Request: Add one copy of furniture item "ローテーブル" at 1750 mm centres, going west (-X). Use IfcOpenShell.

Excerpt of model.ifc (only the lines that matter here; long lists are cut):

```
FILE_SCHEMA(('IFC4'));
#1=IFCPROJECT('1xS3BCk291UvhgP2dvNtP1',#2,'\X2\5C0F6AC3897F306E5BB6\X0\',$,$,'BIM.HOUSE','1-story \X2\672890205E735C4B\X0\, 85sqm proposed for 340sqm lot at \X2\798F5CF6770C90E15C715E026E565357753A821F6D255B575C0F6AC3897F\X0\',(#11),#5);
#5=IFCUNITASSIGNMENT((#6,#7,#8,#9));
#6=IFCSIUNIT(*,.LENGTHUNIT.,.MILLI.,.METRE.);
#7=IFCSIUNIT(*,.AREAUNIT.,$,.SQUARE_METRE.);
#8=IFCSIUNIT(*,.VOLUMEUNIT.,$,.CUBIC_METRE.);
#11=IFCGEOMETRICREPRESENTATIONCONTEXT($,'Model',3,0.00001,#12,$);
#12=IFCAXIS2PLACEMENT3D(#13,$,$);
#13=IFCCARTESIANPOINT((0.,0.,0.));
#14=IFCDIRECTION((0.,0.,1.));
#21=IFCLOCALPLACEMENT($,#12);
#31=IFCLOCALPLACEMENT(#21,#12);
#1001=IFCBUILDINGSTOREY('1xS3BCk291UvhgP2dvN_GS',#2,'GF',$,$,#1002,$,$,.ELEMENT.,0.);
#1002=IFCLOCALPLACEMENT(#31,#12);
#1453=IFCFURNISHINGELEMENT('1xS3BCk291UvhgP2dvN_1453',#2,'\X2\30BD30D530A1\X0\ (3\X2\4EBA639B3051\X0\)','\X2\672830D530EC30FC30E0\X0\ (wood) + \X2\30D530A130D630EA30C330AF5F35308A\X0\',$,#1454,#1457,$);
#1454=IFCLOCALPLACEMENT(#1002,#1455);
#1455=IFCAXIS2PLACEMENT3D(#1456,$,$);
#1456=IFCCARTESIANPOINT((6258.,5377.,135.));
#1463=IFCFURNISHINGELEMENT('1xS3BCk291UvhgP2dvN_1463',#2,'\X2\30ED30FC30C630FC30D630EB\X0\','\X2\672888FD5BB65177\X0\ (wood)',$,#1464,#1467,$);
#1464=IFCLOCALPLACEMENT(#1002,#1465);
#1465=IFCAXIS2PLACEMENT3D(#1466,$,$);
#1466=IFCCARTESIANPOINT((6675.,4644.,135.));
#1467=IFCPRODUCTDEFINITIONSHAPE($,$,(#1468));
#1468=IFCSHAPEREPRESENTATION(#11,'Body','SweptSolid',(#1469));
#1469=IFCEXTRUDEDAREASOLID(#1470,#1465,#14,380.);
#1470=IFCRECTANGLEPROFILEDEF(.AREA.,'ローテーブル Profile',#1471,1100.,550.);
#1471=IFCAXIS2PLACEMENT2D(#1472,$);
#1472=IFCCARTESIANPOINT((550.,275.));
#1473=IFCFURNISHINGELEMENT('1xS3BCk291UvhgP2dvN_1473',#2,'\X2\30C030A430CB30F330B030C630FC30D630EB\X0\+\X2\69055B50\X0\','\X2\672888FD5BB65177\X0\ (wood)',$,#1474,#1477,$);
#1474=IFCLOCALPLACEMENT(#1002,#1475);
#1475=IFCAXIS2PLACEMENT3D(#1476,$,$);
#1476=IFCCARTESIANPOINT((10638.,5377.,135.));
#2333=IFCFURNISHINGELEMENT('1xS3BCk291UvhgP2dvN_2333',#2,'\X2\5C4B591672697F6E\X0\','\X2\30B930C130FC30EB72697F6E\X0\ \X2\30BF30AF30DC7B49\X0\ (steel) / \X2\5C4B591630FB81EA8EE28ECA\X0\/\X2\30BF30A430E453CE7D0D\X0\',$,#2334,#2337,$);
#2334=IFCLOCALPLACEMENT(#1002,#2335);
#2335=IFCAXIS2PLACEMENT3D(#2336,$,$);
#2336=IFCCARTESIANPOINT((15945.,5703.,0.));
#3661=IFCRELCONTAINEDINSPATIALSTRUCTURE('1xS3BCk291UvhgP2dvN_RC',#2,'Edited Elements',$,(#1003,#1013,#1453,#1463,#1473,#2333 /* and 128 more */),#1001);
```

```python
import numpy as np
import ifcopenshell
import ifcopenshell.api.geometry
import ifcopenshell.api.root
import ifcopenshell.util.element
import ifcopenshell.util.placement
import ifcopenshell.util.unit

model = ifcopenshell.open("model.ifc")
unit_scale = ifcopenshell.util.unit.calculate_unit_scale(model)


def reuse_history(source, copy):
    """copy_class also copies each property set's owner history, people and application; keep the originals."""
    for rel in copy.IsDefinedBy:
        if rel.is_a("IfcRelDefinesByProperties") and (history := rel.RelatingPropertyDefinition.OwnerHistory):
            rel.RelatingPropertyDefinition.OwnerHistory = source.OwnerHistory
            ifcopenshell.util.element.remove_deep2(model, history)


source = model.by_guid("1xS3BCk291UvhgP2dvN_1463")
base = ifcopenshell.util.placement.get_local_placement(source.ObjectPlacement)
step = np.array([-1.0, 0.0, 0.0]) * 1.75 / unit_scale

for i in range(1, 2):
    copy = ifcopenshell.api.root.copy_class(model, product=source)
    copy.Representation = ifcopenshell.util.element.copy_deep(
        model, source.Representation, exclude=["IfcGeometricRepresentationContext", "IfcRepresentationMap"]
    )
    reuse_history(source, copy)
    matrix = base.copy()
    matrix[:3, 3] += i * step
    print("added at", matrix[:3, 3].round(3) + 0.0)
    ifcopenshell.api.geometry.edit_object_placement(model, product=copy, matrix=matrix, is_si=False)

model.write("model_v2.ifc")
```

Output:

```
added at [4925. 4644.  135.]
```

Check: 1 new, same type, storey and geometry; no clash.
